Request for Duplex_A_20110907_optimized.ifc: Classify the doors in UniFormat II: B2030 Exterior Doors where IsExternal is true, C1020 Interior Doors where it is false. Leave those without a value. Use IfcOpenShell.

First a look at what the model holds.

```python
import ifcopenshell
import ifcopenshell.util.element

model = ifcopenshell.open("Duplex_A_20110907_optimized.ifc")
print(model.schema)
print("classifications:", [c.Name for c in model.by_type("IfcClassification")])
values = [ifcopenshell.util.element.get_pset(e, "Pset_DoorCommon", "IsExternal") for e in model.by_type("IfcDoor")]
for value in (True, False, None):
    print("IsExternal", value, values.count(value))
```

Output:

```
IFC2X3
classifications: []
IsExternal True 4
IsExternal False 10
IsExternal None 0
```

```python
import ifcopenshell
import ifcopenshell.api.classification
import ifcopenshell.util.element

model = ifcopenshell.open("Duplex_A_20110907_optimized.ifc")

# IFC2X3 requires Source and Edition and has no link from the project to the system.
system = model.create_entity("IfcClassification", Source="ASTM", Edition="E1557", Name="UniFormat II")

doors = model.by_type("IfcDoor")
external = {e: ifcopenshell.util.element.get_pset(e, "Pset_DoorCommon", "IsExternal") for e in doors}
for flag, code, name in ((True, "B2030", "Exterior Doors"), (False, "C1020", "Interior Doors")):
    products = [e for e in doors if external[e] is flag]
    ifcopenshell.api.classification.add_reference(
        model, products=products, classification=system, identification=code, name=name
    )
    print(code, len(products))

model.write("Duplex_A_20110907_optimized_v2.ifc")
```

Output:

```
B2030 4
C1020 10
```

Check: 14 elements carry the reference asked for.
